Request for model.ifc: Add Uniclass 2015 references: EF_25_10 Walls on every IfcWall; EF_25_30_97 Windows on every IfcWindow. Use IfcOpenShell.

First a look at what the model holds.

```python
import ifcopenshell

model = ifcopenshell.open("model.ifc")
print(model.schema)
print("classifications:", [c.Name for c in model.by_type("IfcClassification")])
for ifc_class in ("IfcDoor", "IfcRoof", "IfcStair", "IfcWall", "IfcWindow"):
    print(ifc_class, len(model.by_type(ifc_class)))
```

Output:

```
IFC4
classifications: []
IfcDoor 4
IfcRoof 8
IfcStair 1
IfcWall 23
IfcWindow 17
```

```python
import ifcopenshell
import ifcopenshell.api.classification

model = ifcopenshell.open("model.ifc")

system = ifcopenshell.api.classification.add_classification(model, classification="Uniclass 2015")

codes = {
    "IfcWall": ("EF_25_10", "Walls"),
    "IfcWindow": ("EF_25_30_97", "Windows"),
}
for ifc_class, (code, name) in codes.items():
    products = model.by_type(ifc_class)
    ifcopenshell.api.classification.add_reference(
        model, products=products, classification=system, identification=code, name=name
    )
    print(code, len(products))

model.write("model_edited.ifc")
```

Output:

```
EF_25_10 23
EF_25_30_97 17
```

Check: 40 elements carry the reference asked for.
